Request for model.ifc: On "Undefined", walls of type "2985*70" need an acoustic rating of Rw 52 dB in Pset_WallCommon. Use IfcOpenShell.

First a look at what the model holds.

```python
import ifcopenshell
import ifcopenshell.util.element

model = ifcopenshell.open("model.ifc")
print(model.schema)
storey = next(s for s in model.by_type("IfcBuildingStorey") if s.Name == "Undefined")
walls = [e for e in ifcopenshell.util.element.get_decomposition(storey) if e.is_a("IfcWall")]
seen = {}
for e in walls:
    element_type = ifcopenshell.util.element.get_type(e)
    key = (element_type.Name if element_type != e and element_type else None, ifcopenshell.util.element.get_pset(e, "Pset_WallCommon", "AcousticRating"))
    seen[key] = seen.get(key, 0) + 1
for (name, value), count in sorted(seen.items(), key=str):
    print(count, "x", name, "|", value)
```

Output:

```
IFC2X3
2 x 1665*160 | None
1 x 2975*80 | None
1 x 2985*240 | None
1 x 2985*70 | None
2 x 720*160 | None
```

```python
import ifcopenshell
import ifcopenshell.api.pset
import ifcopenshell.util.element

model = ifcopenshell.open("model.ifc")

storey = next(s for s in model.by_type("IfcBuildingStorey") if s.Name == "Undefined")
walls = [e for e in ifcopenshell.util.element.get_decomposition(storey) if e.is_a("IfcWall")]

count = 0
for e in walls:
    element_type = ifcopenshell.util.element.get_type(e)
    if element_type in (None, e) or element_type.Name != "2985*70":
        continue
    # add_pset returns the element's existing set when there is one.
    pset = ifcopenshell.api.pset.add_pset(model, product=e, name="Pset_WallCommon")
    ifcopenshell.api.pset.edit_pset(model, pset=pset, properties={"AcousticRating": "Rw 52 dB"})
    count += 1

print(count, "walls updated")

model.write("model_updated.ifc")
```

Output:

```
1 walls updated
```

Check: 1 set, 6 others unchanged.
